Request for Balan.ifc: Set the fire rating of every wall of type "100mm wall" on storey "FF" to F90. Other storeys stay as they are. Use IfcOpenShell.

First a look at what the model holds.

```python
import ifcopenshell
import ifcopenshell.util.element

model = ifcopenshell.open("Balan.ifc")
print(model.schema)
storey = next(s for s in model.by_type("IfcBuildingStorey") if s.Name == "FF")
walls = [e for e in ifcopenshell.util.element.get_decomposition(storey) if e.is_a("IfcWall")]
seen = {}
for e in walls:
    element_type = ifcopenshell.util.element.get_type(e)
    key = (element_type.Name if element_type != e and element_type else None, ifcopenshell.util.element.get_pset(e, "Pset_WallCommon", "FireRating"))
    seen[key] = seen.get(key, 0) + 1
for (name, value), count in sorted(seen.items(), key=str):
    print(count, "x", name, "|", value)
```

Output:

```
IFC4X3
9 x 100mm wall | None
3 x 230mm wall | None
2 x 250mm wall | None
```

```python
import ifcopenshell
import ifcopenshell.api.pset
import ifcopenshell.util.element

model = ifcopenshell.open("Balan.ifc")

storey = next(s for s in model.by_type("IfcBuildingStorey") if s.Name == "FF")
walls = [e for e in ifcopenshell.util.element.get_decomposition(storey) if e.is_a("IfcWall")]

count = 0
for e in walls:
    element_type = ifcopenshell.util.element.get_type(e)
    if element_type in (None, e) or element_type.Name != "100mm wall":
        continue
    # add_pset returns the element's existing set when there is one.
    pset = ifcopenshell.api.pset.add_pset(model, product=e, name="Pset_WallCommon")
    ifcopenshell.api.pset.edit_pset(model, pset=pset, properties={"FireRating": "F90"})
    count += 1

print(count, "walls updated")

model.write("Balan_updated.ifc")
```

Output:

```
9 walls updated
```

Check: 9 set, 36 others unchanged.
